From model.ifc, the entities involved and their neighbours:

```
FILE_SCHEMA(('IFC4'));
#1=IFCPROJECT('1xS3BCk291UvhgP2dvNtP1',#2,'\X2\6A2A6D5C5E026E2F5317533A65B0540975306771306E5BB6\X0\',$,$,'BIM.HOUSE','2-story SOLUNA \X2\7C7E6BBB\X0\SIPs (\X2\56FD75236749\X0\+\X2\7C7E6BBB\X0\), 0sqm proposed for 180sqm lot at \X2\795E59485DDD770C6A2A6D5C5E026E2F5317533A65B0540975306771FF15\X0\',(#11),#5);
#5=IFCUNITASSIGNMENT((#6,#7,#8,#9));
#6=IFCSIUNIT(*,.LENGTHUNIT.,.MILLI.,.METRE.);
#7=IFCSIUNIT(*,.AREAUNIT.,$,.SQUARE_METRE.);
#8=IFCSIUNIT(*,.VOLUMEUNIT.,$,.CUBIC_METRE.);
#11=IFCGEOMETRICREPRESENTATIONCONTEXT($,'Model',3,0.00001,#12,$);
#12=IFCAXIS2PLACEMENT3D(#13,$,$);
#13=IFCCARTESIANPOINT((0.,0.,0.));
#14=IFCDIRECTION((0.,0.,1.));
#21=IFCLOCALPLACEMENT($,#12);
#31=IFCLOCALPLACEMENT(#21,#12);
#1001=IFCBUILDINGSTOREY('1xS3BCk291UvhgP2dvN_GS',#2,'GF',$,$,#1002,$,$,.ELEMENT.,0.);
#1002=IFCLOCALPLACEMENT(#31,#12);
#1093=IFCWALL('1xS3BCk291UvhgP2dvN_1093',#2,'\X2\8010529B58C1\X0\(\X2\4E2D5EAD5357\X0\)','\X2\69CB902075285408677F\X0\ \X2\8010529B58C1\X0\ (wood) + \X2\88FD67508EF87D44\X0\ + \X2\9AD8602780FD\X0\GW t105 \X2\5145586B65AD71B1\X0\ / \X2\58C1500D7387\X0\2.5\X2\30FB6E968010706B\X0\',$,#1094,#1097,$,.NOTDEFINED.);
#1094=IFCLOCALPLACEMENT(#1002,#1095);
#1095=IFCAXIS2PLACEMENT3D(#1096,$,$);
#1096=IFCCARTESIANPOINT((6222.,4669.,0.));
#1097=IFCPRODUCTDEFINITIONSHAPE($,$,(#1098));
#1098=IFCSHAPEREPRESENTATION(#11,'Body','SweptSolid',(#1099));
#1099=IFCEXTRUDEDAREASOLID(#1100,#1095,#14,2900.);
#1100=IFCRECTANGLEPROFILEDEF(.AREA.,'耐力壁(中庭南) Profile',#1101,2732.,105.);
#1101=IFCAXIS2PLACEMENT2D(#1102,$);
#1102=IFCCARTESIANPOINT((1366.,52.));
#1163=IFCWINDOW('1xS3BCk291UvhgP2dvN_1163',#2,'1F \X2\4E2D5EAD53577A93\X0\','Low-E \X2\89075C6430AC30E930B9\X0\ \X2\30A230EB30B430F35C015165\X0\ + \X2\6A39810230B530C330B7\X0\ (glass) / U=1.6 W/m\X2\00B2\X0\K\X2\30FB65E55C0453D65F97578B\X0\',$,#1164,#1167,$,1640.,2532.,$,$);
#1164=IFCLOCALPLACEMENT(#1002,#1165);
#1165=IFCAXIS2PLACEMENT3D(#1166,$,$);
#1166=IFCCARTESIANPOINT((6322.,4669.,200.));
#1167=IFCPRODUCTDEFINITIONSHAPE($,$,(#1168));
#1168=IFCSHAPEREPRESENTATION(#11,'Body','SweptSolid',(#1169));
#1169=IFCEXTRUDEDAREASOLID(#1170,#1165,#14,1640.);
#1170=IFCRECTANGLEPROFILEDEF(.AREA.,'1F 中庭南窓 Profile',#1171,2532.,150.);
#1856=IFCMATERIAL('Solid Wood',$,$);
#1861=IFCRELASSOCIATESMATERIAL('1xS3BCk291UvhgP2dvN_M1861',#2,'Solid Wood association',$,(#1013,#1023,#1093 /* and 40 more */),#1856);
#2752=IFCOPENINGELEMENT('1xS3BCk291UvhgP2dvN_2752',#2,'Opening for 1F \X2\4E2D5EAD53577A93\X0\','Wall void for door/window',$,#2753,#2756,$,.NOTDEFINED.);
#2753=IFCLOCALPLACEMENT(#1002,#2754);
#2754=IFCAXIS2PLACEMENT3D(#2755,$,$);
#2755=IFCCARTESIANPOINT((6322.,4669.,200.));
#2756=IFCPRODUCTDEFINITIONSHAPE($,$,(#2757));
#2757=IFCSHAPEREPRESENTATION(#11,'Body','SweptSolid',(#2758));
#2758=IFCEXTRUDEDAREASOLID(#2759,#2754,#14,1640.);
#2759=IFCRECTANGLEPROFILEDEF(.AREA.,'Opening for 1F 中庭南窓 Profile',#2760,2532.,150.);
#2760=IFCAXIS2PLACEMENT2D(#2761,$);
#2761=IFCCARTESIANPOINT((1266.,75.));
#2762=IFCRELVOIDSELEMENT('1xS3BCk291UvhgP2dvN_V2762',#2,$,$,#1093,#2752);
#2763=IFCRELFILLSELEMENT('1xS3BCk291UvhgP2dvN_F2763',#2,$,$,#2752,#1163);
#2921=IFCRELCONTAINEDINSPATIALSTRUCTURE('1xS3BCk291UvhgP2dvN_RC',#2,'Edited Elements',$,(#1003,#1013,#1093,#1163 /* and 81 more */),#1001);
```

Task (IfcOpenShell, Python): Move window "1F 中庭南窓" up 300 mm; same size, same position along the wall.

```python
import numpy as np
import ifcopenshell
import ifcopenshell.api.geometry
import ifcopenshell.util.placement
import ifcopenshell.util.unit

model = ifcopenshell.open("model.ifc")
unit_scale = ifcopenshell.util.unit.calculate_unit_scale(model)

window = model.by_id(1163)
opening = window.FillsVoids[0].RelatingOpeningElement
dz = 300.0

shift = np.array([0.0, 0.0, dz])
# The window is not placed relative to its opening, so move both.
for product in (opening, window):
    matrix = ifcopenshell.util.placement.get_local_placement(product.ObjectPlacement)
    matrix[:3, 3] += shift
    ifcopenshell.api.geometry.edit_object_placement(model, product=product, matrix=matrix, is_si=False)

print(f"moved by {dz * unit_scale:+.3f} m")

model.write("model_v2.ifc")
```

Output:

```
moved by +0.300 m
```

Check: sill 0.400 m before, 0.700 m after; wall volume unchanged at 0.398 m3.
